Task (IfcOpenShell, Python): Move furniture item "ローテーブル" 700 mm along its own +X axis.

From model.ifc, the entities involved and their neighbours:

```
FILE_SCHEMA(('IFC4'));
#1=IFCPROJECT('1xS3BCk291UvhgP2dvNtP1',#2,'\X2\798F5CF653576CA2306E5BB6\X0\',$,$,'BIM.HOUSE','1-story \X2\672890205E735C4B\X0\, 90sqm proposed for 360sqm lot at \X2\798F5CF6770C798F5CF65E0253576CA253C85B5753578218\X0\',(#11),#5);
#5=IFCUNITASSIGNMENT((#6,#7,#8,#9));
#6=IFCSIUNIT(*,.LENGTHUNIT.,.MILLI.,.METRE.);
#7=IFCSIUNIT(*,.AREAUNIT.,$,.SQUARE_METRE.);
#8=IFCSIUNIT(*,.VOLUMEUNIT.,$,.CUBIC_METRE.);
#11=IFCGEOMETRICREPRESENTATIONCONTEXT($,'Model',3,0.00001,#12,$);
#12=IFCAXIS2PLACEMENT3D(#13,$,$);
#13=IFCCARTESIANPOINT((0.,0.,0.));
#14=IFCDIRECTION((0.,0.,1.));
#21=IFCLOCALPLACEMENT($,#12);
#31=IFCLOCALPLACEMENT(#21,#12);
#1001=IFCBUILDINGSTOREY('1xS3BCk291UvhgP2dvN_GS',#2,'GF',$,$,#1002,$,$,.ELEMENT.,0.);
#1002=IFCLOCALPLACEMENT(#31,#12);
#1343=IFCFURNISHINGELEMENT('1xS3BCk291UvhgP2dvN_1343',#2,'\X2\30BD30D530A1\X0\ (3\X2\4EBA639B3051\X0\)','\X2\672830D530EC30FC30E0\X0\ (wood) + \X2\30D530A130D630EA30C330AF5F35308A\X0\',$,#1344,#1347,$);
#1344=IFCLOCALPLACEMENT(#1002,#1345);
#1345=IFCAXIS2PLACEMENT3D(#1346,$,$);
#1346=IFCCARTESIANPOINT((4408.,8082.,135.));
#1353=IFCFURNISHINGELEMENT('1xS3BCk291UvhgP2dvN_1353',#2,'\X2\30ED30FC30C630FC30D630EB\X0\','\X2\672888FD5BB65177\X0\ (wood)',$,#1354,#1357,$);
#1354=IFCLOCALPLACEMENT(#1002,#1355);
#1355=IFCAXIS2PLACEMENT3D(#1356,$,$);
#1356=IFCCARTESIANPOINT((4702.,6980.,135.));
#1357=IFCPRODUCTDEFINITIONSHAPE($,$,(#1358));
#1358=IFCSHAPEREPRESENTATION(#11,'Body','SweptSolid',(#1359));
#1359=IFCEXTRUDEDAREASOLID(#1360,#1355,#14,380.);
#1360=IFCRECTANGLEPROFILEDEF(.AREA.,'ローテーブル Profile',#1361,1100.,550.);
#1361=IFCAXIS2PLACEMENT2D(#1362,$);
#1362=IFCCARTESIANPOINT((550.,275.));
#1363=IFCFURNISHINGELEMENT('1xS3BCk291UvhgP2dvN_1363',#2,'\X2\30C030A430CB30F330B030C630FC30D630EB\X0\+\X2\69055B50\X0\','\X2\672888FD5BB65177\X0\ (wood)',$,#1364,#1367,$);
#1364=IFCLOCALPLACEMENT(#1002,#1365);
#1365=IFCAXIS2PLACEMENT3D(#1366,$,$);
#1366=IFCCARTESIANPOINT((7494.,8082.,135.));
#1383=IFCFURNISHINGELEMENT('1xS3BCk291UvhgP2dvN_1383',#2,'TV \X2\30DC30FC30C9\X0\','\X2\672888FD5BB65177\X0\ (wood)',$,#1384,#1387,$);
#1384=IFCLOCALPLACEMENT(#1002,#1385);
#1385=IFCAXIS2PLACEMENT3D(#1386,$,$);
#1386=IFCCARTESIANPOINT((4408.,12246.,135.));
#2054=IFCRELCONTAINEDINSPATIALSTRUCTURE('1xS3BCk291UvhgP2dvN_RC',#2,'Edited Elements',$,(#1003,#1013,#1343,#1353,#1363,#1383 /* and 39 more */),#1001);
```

```python
import ifcopenshell
import ifcopenshell.api.geometry
import ifcopenshell.util.placement
import ifcopenshell.util.unit

model = ifcopenshell.open("model.ifc")
unit_scale = ifcopenshell.util.unit.calculate_unit_scale(model)

item = model.by_guid("1xS3BCk291UvhgP2dvN_1353")
matrix = ifcopenshell.util.placement.get_local_placement(item.ObjectPlacement)
matrix[:3, 3] += matrix[:3, 0] * 0.7 / unit_scale
ifcopenshell.api.geometry.edit_object_placement(model, product=item, matrix=matrix, is_si=False)

print(ifcopenshell.util.placement.get_local_placement(item.ObjectPlacement).round(3) + 0.0)

model.write("model_edited.ifc")
```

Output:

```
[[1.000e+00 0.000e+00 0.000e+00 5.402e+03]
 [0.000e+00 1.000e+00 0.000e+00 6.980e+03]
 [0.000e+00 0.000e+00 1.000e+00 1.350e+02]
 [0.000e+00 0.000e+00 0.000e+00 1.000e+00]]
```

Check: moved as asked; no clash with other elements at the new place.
